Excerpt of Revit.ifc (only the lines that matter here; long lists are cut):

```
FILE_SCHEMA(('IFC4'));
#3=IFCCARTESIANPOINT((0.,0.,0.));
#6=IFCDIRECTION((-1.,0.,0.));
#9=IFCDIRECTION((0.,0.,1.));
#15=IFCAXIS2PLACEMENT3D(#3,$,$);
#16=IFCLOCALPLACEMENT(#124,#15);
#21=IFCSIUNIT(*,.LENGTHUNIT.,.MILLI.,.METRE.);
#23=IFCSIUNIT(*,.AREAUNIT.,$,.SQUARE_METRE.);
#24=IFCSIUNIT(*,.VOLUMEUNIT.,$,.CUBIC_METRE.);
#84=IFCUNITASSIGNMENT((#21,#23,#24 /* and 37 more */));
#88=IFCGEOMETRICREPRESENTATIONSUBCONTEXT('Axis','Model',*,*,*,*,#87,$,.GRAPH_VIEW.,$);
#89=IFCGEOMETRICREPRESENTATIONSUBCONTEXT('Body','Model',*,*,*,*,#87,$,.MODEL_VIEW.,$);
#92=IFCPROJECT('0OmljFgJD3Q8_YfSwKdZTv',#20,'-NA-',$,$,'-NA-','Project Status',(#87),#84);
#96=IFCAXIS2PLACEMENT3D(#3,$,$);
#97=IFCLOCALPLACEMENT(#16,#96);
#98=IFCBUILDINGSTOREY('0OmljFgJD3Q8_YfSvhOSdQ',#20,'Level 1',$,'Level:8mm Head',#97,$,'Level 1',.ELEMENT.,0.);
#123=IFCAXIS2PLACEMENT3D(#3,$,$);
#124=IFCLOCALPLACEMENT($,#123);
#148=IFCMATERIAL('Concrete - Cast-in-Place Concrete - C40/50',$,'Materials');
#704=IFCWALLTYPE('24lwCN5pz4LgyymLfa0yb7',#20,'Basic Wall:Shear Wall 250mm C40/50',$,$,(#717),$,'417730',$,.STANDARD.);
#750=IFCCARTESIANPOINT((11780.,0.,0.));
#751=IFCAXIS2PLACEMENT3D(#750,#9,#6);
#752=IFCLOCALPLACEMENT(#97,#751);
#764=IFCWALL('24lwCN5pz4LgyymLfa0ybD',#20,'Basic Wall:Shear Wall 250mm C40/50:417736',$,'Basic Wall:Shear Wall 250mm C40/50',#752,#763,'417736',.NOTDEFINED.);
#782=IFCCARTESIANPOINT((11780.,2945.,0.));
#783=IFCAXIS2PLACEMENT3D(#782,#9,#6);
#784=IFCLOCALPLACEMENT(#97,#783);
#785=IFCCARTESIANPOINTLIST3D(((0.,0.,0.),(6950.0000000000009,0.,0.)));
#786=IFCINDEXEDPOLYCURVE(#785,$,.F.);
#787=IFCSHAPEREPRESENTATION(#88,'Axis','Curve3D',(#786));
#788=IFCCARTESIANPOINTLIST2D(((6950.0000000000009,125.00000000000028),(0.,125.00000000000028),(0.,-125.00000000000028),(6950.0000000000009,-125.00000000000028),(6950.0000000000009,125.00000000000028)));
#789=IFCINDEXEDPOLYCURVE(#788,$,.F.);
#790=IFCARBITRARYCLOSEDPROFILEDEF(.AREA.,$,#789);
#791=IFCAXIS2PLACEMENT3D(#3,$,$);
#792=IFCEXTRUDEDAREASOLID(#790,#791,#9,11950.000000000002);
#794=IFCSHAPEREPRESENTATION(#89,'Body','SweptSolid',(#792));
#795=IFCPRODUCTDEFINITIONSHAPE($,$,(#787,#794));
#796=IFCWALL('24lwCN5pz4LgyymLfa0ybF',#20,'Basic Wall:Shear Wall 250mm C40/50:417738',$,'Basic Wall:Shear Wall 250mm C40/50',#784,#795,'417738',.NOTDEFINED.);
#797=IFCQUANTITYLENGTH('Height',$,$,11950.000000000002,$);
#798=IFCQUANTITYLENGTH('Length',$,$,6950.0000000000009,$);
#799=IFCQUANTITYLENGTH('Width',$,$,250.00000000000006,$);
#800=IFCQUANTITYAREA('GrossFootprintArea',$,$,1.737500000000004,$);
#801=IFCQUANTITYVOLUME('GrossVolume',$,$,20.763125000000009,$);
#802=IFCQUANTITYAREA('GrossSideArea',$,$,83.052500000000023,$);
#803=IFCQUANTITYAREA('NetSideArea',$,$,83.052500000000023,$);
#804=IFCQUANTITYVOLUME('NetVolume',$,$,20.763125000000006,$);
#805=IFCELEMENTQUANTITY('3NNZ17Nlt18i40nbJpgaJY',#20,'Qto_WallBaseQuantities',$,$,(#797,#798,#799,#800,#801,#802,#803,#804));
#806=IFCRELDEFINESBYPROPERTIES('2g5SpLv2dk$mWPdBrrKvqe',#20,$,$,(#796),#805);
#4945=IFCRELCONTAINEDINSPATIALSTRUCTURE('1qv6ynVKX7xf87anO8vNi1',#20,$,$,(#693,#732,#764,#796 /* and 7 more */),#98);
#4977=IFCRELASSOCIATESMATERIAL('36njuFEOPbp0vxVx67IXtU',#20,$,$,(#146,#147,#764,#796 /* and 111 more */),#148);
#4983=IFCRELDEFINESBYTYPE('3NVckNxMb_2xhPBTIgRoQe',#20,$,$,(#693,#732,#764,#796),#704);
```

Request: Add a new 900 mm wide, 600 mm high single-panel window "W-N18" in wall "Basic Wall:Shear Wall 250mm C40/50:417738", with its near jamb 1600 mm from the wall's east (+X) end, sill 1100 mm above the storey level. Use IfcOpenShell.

```python
import numpy as np
import ifcopenshell
import ifcopenshell.api.feature
import ifcopenshell.api.geometry
import ifcopenshell.api.pset
import ifcopenshell.api.root
import ifcopenshell.api.spatial
import ifcopenshell.geom
import ifcopenshell.util.element
import ifcopenshell.util.placement
import ifcopenshell.util.representation
import ifcopenshell.util.shape
import ifcopenshell.util.unit

model = ifcopenshell.open("Revit.ifc")
unit_scale = ifcopenshell.util.unit.calculate_unit_scale(model)
area_scale = ifcopenshell.util.unit.calculate_unit_scale(model, "AREAUNIT")
volume_scale = ifcopenshell.util.unit.calculate_unit_scale(model, "VOLUMEUNIT")
settings = ifcopenshell.geom.settings()


def volume(element):
    """Net volume in cubic metres, openings subtracted."""
    shape = ifcopenshell.geom.create_shape(settings, element)
    return ifcopenshell.util.shape.get_volume(shape.geometry)


wall = model.by_id(796)
storey = ifcopenshell.util.element.get_container(wall, ifc_class="IfcBuildingStorey")
context = ifcopenshell.util.representation.get_context(model, "Model", "Body", "MODEL_VIEW")
before = volume(wall)

width, height, from_end, sill = 0.9, 0.6, 1.6, 1.1  # metres

# The wall runs along its own X axis, and the end named is its -X end.
wall_shape = ifcopenshell.geom.create_shape(settings, wall)
x, y, z = ifcopenshell.util.shape.get_vertices(wall_shape.geometry).T
start = x.min() + from_end
face, thickness = float(y.min()), float(y.max() - y.min())
wall_matrix = ifcopenshell.util.placement.get_local_placement(wall.ObjectPlacement)
level = ifcopenshell.util.placement.get_local_placement(storey.ObjectPlacement)[2, 3]


def in_wall(x, y):
    """Placement at x, y metres in the wall's axes, at sill height."""
    matrix = wall_matrix.copy()
    matrix[:, 3] = wall_matrix @ np.array([x / unit_scale, y / unit_scale, 0.0, 1.0])
    matrix[2, 3] = level + sill / unit_scale
    return matrix


# Opening: a box that overshoots both wall faces by 50 mm.
opening = ifcopenshell.api.root.create_entity(model, ifc_class="IfcOpeningElement", predefined_type="OPENING")
box = ifcopenshell.api.geometry.add_wall_representation(
    model, context=context, length=width, height=height, thickness=thickness + 0.1
)
ifcopenshell.api.geometry.assign_representation(model, product=opening, representation=box)
ifcopenshell.api.geometry.edit_object_placement(model, product=opening, matrix=in_wall(start, face - 0.05), is_si=False)
ifcopenshell.api.feature.add_feature(model, feature=opening, element=wall)

window = ifcopenshell.api.root.create_entity(model, ifc_class="IfcWindow", name="W-N18", predefined_type="WINDOW")
window.OverallWidth, window.OverallHeight = width / unit_scale, height / unit_scale
window.PartitioningType = "SINGLE_PANEL"
body = ifcopenshell.api.geometry.add_window_representation(
    model,
    context=context,
    overall_width=window.OverallWidth,
    overall_height=window.OverallHeight,
    partition_type="SINGLE_PANEL",
)
ifcopenshell.api.geometry.assign_representation(model, product=window, representation=body)
ifcopenshell.api.spatial.assign_container(model, products=[window], relating_structure=storey)
ifcopenshell.api.feature.add_filling(model, opening=opening, element=window)

# Centre the window in the wall's thickness.
ifcopenshell.api.geometry.edit_object_placement(model, product=window, matrix=in_wall(start, face), is_si=False)
window_shape = ifcopenshell.geom.create_shape(settings, window)
depth = ifcopenshell.util.shape.get_vertices(window_shape.geometry)[:, 1]
offset = face + thickness / 2 - (depth.min() + depth.max()) / 2
ifcopenshell.api.geometry.edit_object_placement(model, product=window, matrix=in_wall(start, offset), is_si=False)

after = volume(wall)

# Update the wall's stored quantities.
qto = model.by_id(ifcopenshell.util.element.get_pset(wall, "Qto_WallBaseQuantities", should_inherit=False)["id"])
ifcopenshell.api.pset.edit_qto(model, qto=qto, properties={
    "NetSideArea": after / thickness / area_scale,
    "NetVolume": after / volume_scale,
})

print(f"wall volume {before:.3f} -> {after:.3f} m3")

model.write("Revit-out.ifc")
```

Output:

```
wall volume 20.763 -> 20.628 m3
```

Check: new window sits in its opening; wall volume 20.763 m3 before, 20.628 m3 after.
